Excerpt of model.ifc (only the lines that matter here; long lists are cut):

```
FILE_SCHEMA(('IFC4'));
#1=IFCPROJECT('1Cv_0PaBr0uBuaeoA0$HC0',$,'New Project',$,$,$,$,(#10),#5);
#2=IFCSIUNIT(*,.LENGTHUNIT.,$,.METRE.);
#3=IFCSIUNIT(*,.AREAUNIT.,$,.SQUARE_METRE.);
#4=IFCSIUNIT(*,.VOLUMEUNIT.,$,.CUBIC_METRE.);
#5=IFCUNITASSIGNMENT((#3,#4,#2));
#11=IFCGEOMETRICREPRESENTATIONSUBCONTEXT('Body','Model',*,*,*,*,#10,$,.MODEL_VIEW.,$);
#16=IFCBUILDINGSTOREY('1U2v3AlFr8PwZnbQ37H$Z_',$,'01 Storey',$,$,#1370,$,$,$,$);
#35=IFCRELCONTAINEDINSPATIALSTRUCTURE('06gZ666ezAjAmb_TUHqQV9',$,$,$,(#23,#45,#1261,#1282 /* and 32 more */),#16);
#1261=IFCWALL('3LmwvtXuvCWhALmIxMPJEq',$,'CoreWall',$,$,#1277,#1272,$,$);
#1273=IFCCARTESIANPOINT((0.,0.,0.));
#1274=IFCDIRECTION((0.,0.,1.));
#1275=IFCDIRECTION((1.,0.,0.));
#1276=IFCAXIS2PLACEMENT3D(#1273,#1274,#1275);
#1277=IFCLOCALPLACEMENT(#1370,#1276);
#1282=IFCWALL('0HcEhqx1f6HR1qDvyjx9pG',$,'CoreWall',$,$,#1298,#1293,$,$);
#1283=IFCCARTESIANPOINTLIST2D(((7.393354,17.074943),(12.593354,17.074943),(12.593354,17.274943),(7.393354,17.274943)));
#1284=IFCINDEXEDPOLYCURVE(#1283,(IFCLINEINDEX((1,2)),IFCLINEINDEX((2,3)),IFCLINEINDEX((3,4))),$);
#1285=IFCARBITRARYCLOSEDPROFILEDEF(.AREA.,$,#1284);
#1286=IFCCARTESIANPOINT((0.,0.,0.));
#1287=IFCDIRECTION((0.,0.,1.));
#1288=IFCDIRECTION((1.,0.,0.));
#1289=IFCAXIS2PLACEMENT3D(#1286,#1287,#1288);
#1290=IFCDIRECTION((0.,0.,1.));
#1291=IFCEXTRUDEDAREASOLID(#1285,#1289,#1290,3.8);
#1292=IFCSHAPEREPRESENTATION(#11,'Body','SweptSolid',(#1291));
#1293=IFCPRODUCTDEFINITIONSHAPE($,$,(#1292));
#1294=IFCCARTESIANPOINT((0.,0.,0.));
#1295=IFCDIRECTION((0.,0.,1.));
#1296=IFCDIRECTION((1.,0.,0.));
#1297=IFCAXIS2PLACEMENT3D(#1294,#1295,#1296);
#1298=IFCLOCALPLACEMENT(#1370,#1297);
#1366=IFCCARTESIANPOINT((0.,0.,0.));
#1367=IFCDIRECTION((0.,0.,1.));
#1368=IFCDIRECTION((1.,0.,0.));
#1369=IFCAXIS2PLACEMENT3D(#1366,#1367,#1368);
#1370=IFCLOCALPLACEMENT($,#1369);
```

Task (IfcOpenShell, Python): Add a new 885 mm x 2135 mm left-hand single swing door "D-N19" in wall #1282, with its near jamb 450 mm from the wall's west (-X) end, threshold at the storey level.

```python
import numpy as np
import ifcopenshell
import ifcopenshell.api.feature
import ifcopenshell.api.geometry
import ifcopenshell.api.root
import ifcopenshell.api.spatial
import ifcopenshell.geom
import ifcopenshell.util.element
import ifcopenshell.util.placement
import ifcopenshell.util.representation
import ifcopenshell.util.shape
import ifcopenshell.util.unit

model = ifcopenshell.open("model.ifc")
unit_scale = ifcopenshell.util.unit.calculate_unit_scale(model)
settings = ifcopenshell.geom.settings()


def volume(element):
    """Net volume in cubic metres, openings subtracted."""
    shape = ifcopenshell.geom.create_shape(settings, element)
    return ifcopenshell.util.shape.get_volume(shape.geometry)


wall = model.by_id(1282)
storey = ifcopenshell.util.element.get_container(wall, ifc_class="IfcBuildingStorey")
context = ifcopenshell.util.representation.get_context(model, "Model", "Body", "MODEL_VIEW")
before = volume(wall)

width, height, from_end, sill = 0.885, 2.135, 0.45, 0.0  # metres

# The wall runs along its own X axis, and the end named is its -X end.
wall_shape = ifcopenshell.geom.create_shape(settings, wall)
x, y, z = ifcopenshell.util.shape.get_vertices(wall_shape.geometry).T
start = x.min() + from_end
face, thickness = float(y.min()), float(y.max() - y.min())
wall_matrix = ifcopenshell.util.placement.get_local_placement(wall.ObjectPlacement)
level = ifcopenshell.util.placement.get_local_placement(storey.ObjectPlacement)[2, 3]


def in_wall(x, y):
    """Placement at x, y metres in the wall's axes, at sill height."""
    matrix = wall_matrix.copy()
    matrix[:, 3] = wall_matrix @ np.array([x / unit_scale, y / unit_scale, 0.0, 1.0])
    matrix[2, 3] = level + sill / unit_scale
    return matrix


# Opening: a box that overshoots both wall faces by 50 mm.
opening = ifcopenshell.api.root.create_entity(model, ifc_class="IfcOpeningElement", predefined_type="OPENING")
box = ifcopenshell.api.geometry.add_wall_representation(
    model, context=context, length=width, height=height, thickness=thickness + 0.1
)
ifcopenshell.api.geometry.assign_representation(model, product=opening, representation=box)
ifcopenshell.api.geometry.edit_object_placement(model, product=opening, matrix=in_wall(start, face - 0.05), is_si=False)
ifcopenshell.api.feature.add_feature(model, feature=opening, element=wall)

door = ifcopenshell.api.root.create_entity(model, ifc_class="IfcDoor", name="D-N19", predefined_type="DOOR")
door.OverallWidth, door.OverallHeight = width / unit_scale, height / unit_scale
door.OperationType = "SINGLE_SWING_LEFT"
body = ifcopenshell.api.geometry.add_door_representation(
    model,
    context=context,
    overall_width=door.OverallWidth,
    overall_height=door.OverallHeight,
    operation_type="SINGLE_SWING_LEFT",
    lining_properties={"LiningDepth": thickness / unit_scale, "ThresholdDepth": thickness / unit_scale},
)
ifcopenshell.api.geometry.assign_representation(model, product=door, representation=body)
ifcopenshell.api.spatial.assign_container(model, products=[door], relating_structure=storey)
ifcopenshell.api.feature.add_filling(model, opening=opening, element=door)

# The lining spans the wall, so the door starts at the wall face.
ifcopenshell.api.geometry.edit_object_placement(model, product=door, matrix=in_wall(start, face), is_si=False)

after = volume(wall)

print(f"wall volume {before:.3f} -> {after:.3f} m3")

model.write("model_edited.ifc")
```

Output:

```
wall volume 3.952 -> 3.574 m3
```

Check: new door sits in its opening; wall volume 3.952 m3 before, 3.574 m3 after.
